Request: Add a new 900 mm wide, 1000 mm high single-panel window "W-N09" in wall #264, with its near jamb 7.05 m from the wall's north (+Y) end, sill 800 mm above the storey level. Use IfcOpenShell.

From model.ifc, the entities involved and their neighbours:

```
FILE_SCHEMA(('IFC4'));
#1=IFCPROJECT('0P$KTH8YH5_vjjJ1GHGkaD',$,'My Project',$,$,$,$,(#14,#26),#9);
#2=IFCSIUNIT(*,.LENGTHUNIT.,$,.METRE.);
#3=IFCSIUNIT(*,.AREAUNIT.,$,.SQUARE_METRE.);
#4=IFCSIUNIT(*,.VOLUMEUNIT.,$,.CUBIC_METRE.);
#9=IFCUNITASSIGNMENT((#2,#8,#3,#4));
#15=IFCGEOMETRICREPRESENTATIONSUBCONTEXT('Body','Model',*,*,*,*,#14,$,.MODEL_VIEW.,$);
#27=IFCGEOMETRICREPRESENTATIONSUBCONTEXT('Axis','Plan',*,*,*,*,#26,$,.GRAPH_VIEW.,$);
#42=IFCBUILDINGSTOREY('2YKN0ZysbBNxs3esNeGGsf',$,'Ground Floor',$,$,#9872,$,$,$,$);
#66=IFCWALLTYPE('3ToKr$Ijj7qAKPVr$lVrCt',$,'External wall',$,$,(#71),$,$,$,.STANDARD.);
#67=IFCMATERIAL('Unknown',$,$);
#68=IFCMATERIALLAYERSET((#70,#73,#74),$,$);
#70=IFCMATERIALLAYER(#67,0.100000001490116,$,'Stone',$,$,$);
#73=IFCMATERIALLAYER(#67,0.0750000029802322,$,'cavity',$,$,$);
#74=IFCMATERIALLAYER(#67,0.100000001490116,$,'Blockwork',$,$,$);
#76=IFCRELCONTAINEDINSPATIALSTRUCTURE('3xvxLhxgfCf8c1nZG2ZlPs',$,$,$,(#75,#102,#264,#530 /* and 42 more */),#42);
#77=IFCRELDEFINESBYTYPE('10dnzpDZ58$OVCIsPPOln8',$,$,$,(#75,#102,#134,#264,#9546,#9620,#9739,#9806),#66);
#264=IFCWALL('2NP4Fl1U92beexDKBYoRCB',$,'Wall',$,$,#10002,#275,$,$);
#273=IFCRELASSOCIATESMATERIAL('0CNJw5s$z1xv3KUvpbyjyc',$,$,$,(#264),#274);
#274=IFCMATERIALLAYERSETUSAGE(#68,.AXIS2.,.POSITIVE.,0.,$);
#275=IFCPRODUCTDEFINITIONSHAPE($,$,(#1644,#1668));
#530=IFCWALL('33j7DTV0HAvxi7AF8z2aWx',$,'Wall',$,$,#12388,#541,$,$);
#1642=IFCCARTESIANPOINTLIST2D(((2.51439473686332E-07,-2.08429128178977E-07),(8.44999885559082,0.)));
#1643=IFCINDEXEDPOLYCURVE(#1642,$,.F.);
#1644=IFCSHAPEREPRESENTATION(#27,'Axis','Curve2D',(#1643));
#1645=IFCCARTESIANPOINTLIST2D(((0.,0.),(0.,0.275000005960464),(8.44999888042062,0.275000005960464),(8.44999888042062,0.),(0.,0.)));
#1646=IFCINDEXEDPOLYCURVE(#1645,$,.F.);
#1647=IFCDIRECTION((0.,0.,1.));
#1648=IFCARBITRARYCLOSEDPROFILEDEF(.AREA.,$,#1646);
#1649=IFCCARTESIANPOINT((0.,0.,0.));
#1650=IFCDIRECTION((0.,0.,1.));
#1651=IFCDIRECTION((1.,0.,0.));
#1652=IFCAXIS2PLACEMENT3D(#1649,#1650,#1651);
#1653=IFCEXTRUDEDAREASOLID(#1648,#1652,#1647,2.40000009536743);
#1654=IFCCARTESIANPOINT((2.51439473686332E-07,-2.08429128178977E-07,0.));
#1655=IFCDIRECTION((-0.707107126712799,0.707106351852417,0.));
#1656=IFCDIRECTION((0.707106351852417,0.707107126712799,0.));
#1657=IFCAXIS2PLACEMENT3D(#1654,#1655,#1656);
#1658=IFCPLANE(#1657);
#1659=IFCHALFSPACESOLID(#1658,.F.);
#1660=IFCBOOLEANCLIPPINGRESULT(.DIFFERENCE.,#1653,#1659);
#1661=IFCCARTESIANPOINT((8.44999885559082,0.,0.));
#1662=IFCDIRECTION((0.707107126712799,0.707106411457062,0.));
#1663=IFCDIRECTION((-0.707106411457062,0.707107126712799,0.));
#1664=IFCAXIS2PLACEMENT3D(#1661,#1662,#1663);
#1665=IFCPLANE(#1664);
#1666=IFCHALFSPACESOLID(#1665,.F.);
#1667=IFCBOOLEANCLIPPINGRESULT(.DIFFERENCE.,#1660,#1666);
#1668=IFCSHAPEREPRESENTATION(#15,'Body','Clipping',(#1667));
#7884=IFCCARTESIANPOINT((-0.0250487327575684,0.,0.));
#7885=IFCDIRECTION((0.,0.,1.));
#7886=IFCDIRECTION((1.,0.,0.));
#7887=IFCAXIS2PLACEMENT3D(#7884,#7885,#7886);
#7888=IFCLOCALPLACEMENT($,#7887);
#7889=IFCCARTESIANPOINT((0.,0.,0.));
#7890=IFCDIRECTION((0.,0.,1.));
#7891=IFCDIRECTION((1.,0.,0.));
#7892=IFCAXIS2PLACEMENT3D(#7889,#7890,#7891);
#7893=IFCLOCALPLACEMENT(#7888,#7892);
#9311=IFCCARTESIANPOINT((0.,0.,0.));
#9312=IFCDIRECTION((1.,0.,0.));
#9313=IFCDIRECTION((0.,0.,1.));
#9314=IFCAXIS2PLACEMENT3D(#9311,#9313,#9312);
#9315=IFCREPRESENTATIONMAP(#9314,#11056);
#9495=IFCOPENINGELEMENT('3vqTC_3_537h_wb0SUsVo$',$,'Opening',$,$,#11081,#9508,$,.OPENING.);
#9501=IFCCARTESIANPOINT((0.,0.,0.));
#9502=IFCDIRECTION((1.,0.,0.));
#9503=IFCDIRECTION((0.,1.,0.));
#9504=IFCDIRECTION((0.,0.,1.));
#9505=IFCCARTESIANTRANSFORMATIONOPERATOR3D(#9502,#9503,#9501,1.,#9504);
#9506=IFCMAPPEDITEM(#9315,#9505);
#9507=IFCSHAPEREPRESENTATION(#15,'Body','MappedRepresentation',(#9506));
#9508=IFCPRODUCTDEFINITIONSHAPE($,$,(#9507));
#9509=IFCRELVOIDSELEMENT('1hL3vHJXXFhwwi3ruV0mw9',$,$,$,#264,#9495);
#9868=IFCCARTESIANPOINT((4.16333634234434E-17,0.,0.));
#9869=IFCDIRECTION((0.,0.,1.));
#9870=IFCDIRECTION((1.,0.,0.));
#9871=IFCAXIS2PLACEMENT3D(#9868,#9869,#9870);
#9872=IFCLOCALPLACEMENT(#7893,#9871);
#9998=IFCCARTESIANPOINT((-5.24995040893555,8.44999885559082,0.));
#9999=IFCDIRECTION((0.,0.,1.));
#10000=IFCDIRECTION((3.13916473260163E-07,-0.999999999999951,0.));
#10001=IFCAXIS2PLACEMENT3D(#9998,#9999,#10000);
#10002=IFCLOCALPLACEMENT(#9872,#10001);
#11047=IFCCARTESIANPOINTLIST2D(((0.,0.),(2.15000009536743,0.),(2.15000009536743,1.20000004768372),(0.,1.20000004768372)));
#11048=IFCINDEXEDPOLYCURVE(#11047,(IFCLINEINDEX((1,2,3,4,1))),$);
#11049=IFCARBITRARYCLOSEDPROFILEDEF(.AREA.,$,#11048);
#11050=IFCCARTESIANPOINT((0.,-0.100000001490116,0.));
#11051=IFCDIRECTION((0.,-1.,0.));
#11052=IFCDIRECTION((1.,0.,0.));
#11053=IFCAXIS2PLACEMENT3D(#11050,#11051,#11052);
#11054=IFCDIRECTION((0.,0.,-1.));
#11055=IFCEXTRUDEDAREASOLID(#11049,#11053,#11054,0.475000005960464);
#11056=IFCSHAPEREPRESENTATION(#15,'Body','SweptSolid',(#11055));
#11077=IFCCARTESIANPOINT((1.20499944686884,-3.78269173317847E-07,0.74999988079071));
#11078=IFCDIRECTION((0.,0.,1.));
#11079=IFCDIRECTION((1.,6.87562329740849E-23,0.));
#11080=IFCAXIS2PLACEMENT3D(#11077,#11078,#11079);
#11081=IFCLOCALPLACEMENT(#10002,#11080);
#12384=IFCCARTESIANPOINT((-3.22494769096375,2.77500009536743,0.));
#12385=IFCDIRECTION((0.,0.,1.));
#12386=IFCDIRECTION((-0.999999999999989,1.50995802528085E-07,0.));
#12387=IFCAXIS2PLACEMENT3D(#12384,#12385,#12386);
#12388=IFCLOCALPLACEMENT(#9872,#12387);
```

```python
import numpy as np
import ifcopenshell
import ifcopenshell.api.feature
import ifcopenshell.api.geometry
import ifcopenshell.api.root
import ifcopenshell.api.spatial
import ifcopenshell.geom
import ifcopenshell.util.element
import ifcopenshell.util.placement
import ifcopenshell.util.representation
import ifcopenshell.util.shape
import ifcopenshell.util.unit

model = ifcopenshell.open("model.ifc")
unit_scale = ifcopenshell.util.unit.calculate_unit_scale(model)
settings = ifcopenshell.geom.settings()


def volume(element):
    """Net volume in cubic metres, openings subtracted."""
    shape = ifcopenshell.geom.create_shape(settings, element)
    return ifcopenshell.util.shape.get_volume(shape.geometry)


wall = model.by_guid("2NP4Fl1U92beexDKBYoRCB")
storey = ifcopenshell.util.element.get_container(wall, ifc_class="IfcBuildingStorey")
context = ifcopenshell.util.representation.get_context(model, "Model", "Body", "MODEL_VIEW")
before = volume(wall)

width, height, from_end, sill = 0.9, 1, 7.05, 0.8  # metres

# The wall runs along its own X axis, and the end named is its -X end.
wall_shape = ifcopenshell.geom.create_shape(settings, wall)
x, y, z = ifcopenshell.util.shape.get_vertices(wall_shape.geometry).T
start = x.min() + from_end
face, thickness = float(y.min()), float(y.max() - y.min())
wall_matrix = ifcopenshell.util.placement.get_local_placement(wall.ObjectPlacement)
level = ifcopenshell.util.placement.get_local_placement(storey.ObjectPlacement)[2, 3]


def in_wall(x, y):
    """Placement at x, y metres in the wall's axes, at sill height."""
    matrix = wall_matrix.copy()
    matrix[:, 3] = wall_matrix @ np.array([x / unit_scale, y / unit_scale, 0.0, 1.0])
    matrix[2, 3] = level + sill / unit_scale
    return matrix


# Opening: a box that overshoots both wall faces by 50 mm.
opening = ifcopenshell.api.root.create_entity(model, ifc_class="IfcOpeningElement", predefined_type="OPENING")
box = ifcopenshell.api.geometry.add_wall_representation(
    model, context=context, length=width, height=height, thickness=thickness + 0.1
)
ifcopenshell.api.geometry.assign_representation(model, product=opening, representation=box)
ifcopenshell.api.geometry.edit_object_placement(model, product=opening, matrix=in_wall(start, face - 0.05), is_si=False)
ifcopenshell.api.feature.add_feature(model, feature=opening, element=wall)

window = ifcopenshell.api.root.create_entity(model, ifc_class="IfcWindow", name="W-N09", predefined_type="WINDOW")
window.OverallWidth, window.OverallHeight = width / unit_scale, height / unit_scale
window.PartitioningType = "SINGLE_PANEL"
body = ifcopenshell.api.geometry.add_window_representation(
    model,
    context=context,
    overall_width=window.OverallWidth,
    overall_height=window.OverallHeight,
    partition_type="SINGLE_PANEL",
)
ifcopenshell.api.geometry.assign_representation(model, product=window, representation=body)
ifcopenshell.api.spatial.assign_container(model, products=[window], relating_structure=storey)
ifcopenshell.api.feature.add_filling(model, opening=opening, element=window)

# Centre the window in the wall's thickness.
ifcopenshell.api.geometry.edit_object_placement(model, product=window, matrix=in_wall(start, face), is_si=False)
window_shape = ifcopenshell.geom.create_shape(settings, window)
depth = ifcopenshell.util.shape.get_vertices(window_shape.geometry)[:, 1]
offset = face + thickness / 2 - (depth.min() + depth.max()) / 2
ifcopenshell.api.geometry.edit_object_placement(model, product=window, matrix=in_wall(start, offset), is_si=False)

after = volume(wall)

print(f"wall volume {before:.3f} -> {after:.3f} m3")

model.write("model_v2.ifc")
```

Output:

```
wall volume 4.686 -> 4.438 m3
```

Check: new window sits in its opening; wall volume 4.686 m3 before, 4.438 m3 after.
